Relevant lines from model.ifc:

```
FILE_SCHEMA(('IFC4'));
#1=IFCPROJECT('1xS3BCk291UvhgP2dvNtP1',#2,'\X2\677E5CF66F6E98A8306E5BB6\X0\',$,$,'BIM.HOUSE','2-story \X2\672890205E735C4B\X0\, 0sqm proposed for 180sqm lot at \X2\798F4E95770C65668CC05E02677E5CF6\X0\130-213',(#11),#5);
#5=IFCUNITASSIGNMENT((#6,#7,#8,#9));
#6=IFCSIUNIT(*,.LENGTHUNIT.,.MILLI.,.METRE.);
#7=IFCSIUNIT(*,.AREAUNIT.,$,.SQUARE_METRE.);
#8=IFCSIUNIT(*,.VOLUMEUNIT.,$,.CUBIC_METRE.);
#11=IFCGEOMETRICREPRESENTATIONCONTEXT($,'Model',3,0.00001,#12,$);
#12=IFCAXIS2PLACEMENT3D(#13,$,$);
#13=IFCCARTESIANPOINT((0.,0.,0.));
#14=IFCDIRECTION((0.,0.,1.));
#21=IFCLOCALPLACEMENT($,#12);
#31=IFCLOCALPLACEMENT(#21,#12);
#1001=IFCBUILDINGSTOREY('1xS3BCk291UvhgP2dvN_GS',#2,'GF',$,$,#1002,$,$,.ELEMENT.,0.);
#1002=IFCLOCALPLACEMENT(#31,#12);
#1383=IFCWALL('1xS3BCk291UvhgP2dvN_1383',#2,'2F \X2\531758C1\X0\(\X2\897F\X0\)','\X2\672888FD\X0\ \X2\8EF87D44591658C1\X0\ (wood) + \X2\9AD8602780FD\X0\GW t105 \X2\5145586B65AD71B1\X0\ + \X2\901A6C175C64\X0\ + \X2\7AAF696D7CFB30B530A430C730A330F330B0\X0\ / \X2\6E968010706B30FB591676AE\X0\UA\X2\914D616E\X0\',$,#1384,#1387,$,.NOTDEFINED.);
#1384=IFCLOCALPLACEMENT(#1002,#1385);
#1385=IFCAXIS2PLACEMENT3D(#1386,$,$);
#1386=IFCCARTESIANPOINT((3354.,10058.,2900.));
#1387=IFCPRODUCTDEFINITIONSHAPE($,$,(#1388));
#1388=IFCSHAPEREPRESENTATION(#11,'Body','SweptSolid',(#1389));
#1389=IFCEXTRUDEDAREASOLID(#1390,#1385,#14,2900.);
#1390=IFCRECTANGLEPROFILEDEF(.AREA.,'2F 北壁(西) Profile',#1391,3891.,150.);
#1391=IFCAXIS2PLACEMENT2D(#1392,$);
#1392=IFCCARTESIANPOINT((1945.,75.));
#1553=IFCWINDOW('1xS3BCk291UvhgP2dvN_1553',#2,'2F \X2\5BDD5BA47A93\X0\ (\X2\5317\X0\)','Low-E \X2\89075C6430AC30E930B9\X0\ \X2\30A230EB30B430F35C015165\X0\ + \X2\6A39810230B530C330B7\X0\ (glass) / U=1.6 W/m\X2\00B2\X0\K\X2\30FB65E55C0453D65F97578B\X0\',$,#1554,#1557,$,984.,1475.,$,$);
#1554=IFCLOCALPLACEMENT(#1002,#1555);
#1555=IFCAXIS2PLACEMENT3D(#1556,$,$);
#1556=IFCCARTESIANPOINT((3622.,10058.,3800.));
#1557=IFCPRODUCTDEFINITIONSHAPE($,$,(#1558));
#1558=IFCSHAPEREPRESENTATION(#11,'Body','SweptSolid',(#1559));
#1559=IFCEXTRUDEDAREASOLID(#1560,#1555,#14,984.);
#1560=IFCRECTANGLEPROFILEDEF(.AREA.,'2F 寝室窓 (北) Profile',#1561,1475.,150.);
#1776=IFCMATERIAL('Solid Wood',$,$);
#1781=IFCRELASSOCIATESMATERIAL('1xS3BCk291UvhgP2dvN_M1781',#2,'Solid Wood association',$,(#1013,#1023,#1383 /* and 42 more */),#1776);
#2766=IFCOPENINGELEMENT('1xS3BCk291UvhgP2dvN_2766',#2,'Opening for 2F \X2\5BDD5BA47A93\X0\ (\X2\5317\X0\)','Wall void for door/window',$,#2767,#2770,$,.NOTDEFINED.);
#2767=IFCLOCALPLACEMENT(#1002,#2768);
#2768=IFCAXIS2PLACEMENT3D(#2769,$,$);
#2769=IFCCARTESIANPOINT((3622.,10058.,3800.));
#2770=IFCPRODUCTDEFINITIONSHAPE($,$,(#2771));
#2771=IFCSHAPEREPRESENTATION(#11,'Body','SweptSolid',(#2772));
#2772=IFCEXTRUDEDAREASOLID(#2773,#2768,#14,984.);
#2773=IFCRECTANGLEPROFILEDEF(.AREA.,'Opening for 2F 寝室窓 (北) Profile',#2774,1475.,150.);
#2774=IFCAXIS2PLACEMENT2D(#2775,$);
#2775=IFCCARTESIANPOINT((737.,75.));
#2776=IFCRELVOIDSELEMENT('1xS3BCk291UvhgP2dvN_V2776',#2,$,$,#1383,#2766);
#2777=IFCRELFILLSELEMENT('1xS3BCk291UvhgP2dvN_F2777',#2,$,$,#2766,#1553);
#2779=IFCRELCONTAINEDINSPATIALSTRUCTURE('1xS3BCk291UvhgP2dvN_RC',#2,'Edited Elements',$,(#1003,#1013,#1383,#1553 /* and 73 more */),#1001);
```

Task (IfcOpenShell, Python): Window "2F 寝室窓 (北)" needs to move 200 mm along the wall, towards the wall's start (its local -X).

```python
import ifcopenshell
import ifcopenshell.api.geometry
import ifcopenshell.util.placement
import ifcopenshell.util.unit

model = ifcopenshell.open("model.ifc")
unit_scale = ifcopenshell.util.unit.calculate_unit_scale(model)

window = model.by_guid("1xS3BCk291UvhgP2dvN_1553")
opening = window.FillsVoids[0].RelatingOpeningElement
wall = opening.VoidsElements[0].RelatingBuildingElement

wall_matrix = ifcopenshell.util.placement.get_local_placement(wall.ObjectPlacement)
shift = wall_matrix[:3, 0] * -0.2 / unit_scale
before = ifcopenshell.util.placement.get_local_placement(window.ObjectPlacement)[:3, 3].copy()

# The window is not placed relative to its opening, so move both.
for product in (opening, window):
    matrix = ifcopenshell.util.placement.get_local_placement(product.ObjectPlacement)
    matrix[:3, 3] += shift
    ifcopenshell.api.geometry.edit_object_placement(model, product=product, matrix=matrix, is_si=False)

after = ifcopenshell.util.placement.get_local_placement(window.ObjectPlacement)[:3, 3]
print("window moved by", (after - before).round(3) + 0.0)

model.write("model_updated.ifc")
```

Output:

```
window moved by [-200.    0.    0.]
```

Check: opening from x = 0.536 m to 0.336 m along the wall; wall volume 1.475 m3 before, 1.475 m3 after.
